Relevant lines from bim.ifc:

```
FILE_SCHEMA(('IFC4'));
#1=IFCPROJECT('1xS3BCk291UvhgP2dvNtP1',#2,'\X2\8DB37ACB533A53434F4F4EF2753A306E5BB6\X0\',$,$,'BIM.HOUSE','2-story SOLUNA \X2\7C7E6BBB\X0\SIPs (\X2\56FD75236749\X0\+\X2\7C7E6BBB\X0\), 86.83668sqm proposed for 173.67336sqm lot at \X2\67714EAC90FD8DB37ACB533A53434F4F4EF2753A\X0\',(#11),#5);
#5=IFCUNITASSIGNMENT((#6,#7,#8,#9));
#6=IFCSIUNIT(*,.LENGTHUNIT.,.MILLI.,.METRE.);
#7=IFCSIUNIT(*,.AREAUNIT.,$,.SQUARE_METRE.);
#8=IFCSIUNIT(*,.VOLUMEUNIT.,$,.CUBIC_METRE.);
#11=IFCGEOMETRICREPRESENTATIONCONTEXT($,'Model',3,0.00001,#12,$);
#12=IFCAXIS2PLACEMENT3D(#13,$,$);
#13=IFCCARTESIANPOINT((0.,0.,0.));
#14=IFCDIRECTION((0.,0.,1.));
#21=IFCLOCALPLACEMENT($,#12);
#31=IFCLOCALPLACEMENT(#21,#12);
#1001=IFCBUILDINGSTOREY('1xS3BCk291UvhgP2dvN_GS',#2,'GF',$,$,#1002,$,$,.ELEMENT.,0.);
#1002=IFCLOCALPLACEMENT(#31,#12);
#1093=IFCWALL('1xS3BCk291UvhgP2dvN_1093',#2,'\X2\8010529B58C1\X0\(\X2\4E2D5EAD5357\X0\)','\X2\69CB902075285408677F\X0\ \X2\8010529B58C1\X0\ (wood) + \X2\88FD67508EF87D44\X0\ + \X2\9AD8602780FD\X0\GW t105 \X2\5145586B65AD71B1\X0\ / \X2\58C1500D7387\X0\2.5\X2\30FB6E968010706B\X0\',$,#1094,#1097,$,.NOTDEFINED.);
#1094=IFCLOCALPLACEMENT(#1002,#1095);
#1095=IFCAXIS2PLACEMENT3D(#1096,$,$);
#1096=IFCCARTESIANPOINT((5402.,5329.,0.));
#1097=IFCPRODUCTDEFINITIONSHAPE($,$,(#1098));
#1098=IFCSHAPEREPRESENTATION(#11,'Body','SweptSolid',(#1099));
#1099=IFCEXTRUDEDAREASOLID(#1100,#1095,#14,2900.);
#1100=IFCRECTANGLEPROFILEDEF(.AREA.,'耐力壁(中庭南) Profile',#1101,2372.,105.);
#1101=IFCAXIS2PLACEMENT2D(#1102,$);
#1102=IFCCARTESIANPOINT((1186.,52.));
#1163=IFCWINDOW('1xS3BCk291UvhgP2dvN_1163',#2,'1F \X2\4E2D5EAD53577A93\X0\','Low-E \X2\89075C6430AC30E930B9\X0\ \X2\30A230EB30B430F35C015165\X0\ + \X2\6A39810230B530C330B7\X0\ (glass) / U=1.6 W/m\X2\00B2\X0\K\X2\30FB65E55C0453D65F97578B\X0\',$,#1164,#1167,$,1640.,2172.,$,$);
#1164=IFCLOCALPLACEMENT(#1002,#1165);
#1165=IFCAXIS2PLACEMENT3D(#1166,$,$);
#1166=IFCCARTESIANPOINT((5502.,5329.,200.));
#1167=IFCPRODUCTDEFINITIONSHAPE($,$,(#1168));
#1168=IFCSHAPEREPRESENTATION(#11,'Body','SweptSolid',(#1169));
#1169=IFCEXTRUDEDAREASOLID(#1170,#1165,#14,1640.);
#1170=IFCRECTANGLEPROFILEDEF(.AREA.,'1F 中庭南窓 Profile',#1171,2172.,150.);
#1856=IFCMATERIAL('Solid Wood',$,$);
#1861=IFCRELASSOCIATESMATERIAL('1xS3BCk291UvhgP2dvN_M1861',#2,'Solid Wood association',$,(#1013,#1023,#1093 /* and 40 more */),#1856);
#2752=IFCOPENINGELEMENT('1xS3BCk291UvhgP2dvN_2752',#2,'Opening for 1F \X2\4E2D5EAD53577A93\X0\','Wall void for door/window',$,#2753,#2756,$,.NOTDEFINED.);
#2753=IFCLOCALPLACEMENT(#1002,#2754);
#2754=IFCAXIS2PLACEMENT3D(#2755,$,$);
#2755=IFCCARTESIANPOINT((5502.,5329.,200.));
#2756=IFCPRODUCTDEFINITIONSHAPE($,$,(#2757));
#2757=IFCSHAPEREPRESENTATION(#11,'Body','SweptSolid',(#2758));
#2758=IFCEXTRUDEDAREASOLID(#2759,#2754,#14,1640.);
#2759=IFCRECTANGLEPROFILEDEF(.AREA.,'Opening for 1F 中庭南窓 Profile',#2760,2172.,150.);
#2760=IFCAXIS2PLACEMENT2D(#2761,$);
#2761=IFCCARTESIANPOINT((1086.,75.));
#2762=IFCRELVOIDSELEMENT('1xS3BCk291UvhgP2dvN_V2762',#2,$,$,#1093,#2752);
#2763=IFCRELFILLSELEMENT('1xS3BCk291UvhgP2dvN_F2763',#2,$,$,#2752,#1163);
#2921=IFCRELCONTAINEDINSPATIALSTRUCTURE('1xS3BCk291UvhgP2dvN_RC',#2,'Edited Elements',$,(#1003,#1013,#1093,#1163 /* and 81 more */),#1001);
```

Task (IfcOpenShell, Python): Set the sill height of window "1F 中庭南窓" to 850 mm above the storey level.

```python
import numpy as np
import ifcopenshell
import ifcopenshell.api.geometry
import ifcopenshell.geom
import ifcopenshell.util.element
import ifcopenshell.util.placement
import ifcopenshell.util.shape
import ifcopenshell.util.unit

model = ifcopenshell.open("bim.ifc")
unit_scale = ifcopenshell.util.unit.calculate_unit_scale(model)

window = model.by_guid("1xS3BCk291UvhgP2dvN_1163")
opening = window.FillsVoids[0].RelatingOpeningElement
storey = ifcopenshell.util.element.get_container(window, ifc_class="IfcBuildingStorey")
level = ifcopenshell.util.placement.get_local_placement(storey.ObjectPlacement)[2, 3]

# The opening's origin need not be at the sill, so measure its lowest point.
shape = ifcopenshell.geom.create_shape(ifcopenshell.geom.settings(), opening)
bottom = ifcopenshell.util.shape.get_shape_bottom_elevation(shape, shape.geometry) / unit_scale
dz = level + 0.85 / unit_scale - bottom

shift = np.array([0.0, 0.0, dz])
# The window is not placed relative to its opening, so move both.
for product in (opening, window):
    matrix = ifcopenshell.util.placement.get_local_placement(product.ObjectPlacement)
    matrix[:3, 3] += shift
    ifcopenshell.api.geometry.edit_object_placement(model, product=product, matrix=matrix, is_si=False)

print(f"moved by {dz * unit_scale:+.3f} m")

model.write("bim_rev.ifc")
```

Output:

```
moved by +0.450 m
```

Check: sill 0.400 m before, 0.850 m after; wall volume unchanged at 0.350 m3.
